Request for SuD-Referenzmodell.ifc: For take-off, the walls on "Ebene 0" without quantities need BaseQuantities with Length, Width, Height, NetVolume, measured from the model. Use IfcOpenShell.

First a look at what the model holds.

```python
import ifcopenshell
import ifcopenshell.util.element
import ifcopenshell.util.unit

model = ifcopenshell.open("SuD-Referenzmodell.ifc")
print(model.schema)
for unit_type in ("LENGTHUNIT", "AREAUNIT", "VOLUMEUNIT"):
    print(unit_type, ifcopenshell.util.unit.calculate_unit_scale(model, unit_type))
storey = next(s for s in model.by_type("IfcBuildingStorey") if s.Name == "Ebene 0")
walls = [e for e in ifcopenshell.util.element.get_decomposition(storey) if e.is_a("IfcWall")]
for e in sorted(walls, key=lambda e: e.id()):
    print(e.id(), e.is_a(), e.Name, list(ifcopenshell.util.element.get_psets(e, qtos_only=True)), sep=" | ")
```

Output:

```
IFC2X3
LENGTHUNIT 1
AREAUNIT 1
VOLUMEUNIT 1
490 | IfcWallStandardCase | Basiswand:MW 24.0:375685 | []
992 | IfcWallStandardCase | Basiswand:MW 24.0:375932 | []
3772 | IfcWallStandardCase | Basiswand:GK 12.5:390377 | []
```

```python
import ifcopenshell
import ifcopenshell.api.pset
import ifcopenshell.geom
import ifcopenshell.util.element
import ifcopenshell.util.shape
import ifcopenshell.util.unit

model = ifcopenshell.open("SuD-Referenzmodell.ifc")
unit_scale = ifcopenshell.util.unit.calculate_unit_scale(model)
volume_scale = ifcopenshell.util.unit.calculate_unit_scale(model, "VOLUMEUNIT")
settings = ifcopenshell.geom.settings()

storey = next(s for s in model.by_type("IfcBuildingStorey") if s.Name == "Ebene 0")
walls = [e for e in ifcopenshell.util.element.get_decomposition(storey) if e.is_a("IfcWall")]

for e in sorted(walls, key=lambda e: e.id()):
    if ifcopenshell.util.element.get_psets(e, qtos_only=True, should_inherit=False):
        continue
    # Geometry comes back in metres, in the element's own axes.
    shape = ifcopenshell.geom.create_shape(settings, e)
    values = {
        "Length": ifcopenshell.util.shape.get_x(shape.geometry) / unit_scale,
        "Width": ifcopenshell.util.shape.get_y(shape.geometry) / unit_scale,
        "Height": ifcopenshell.util.shape.get_z(shape.geometry) / unit_scale,
        "NetVolume": ifcopenshell.util.shape.get_volume(shape.geometry) / volume_scale,
    }
    qto = ifcopenshell.api.pset.add_qto(model, product=e, name="BaseQuantities")
    ifcopenshell.api.pset.edit_qto(model, qto=qto, properties=values)
    print(e.id(), {k: round(v, 3) for k, v in values.items()})

model.write("SuD-Referenzmodell_edited.ifc")
```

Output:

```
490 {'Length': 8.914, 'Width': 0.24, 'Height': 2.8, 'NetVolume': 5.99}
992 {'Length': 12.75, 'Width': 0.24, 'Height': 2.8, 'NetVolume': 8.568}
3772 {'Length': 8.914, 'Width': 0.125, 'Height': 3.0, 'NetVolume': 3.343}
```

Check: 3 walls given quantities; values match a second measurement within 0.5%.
